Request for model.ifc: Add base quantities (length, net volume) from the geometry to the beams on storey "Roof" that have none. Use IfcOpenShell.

First a look at what the model holds.

```python
import ifcopenshell
import ifcopenshell.util.element
import ifcopenshell.util.unit

model = ifcopenshell.open("model.ifc")
print(model.schema)
for unit_type in ("LENGTHUNIT", "AREAUNIT", "VOLUMEUNIT"):
    print(unit_type, ifcopenshell.util.unit.calculate_unit_scale(model, unit_type))
storey = next(s for s in model.by_type("IfcBuildingStorey") if s.Name == "Roof")
beams = [e for e in ifcopenshell.util.element.get_decomposition(storey) if e.is_a("IfcBeam")]
for e in sorted(beams, key=lambda e: e.id()):
    print(e.id(), e.is_a(), e.Name, list(ifcopenshell.util.element.get_psets(e, qtos_only=True)), sep=" | ")
```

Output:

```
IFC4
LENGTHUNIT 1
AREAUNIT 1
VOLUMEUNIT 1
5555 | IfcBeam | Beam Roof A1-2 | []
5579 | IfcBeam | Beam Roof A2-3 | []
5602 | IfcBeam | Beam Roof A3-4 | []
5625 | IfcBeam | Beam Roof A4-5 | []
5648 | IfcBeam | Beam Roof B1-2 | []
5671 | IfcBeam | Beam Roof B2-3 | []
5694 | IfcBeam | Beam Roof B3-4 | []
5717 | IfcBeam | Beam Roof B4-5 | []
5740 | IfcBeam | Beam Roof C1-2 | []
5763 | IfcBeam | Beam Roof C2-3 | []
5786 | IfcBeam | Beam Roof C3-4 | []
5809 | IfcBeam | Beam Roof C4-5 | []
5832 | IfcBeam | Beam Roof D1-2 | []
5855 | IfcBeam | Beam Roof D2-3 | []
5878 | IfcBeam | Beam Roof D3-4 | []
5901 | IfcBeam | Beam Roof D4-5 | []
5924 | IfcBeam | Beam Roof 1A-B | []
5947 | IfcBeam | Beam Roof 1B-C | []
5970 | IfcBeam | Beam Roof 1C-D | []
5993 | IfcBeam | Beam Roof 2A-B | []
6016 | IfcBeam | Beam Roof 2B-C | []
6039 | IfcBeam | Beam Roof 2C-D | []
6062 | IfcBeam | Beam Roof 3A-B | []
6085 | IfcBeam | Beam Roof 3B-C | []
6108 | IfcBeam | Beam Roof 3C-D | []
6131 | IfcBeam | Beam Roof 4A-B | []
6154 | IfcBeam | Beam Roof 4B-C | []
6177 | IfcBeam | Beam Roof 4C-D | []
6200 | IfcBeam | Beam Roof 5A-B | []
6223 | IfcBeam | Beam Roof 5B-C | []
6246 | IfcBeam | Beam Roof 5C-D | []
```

```python
import ifcopenshell
import ifcopenshell.api.pset
import ifcopenshell.geom
import ifcopenshell.util.element
import ifcopenshell.util.shape
import ifcopenshell.util.unit

model = ifcopenshell.open("model.ifc")
unit_scale = ifcopenshell.util.unit.calculate_unit_scale(model)
volume_scale = ifcopenshell.util.unit.calculate_unit_scale(model, "VOLUMEUNIT")
settings = ifcopenshell.geom.settings()

storey = next(s for s in model.by_type("IfcBuildingStorey") if s.Name == "Roof")
beams = [e for e in ifcopenshell.util.element.get_decomposition(storey) if e.is_a("IfcBeam")]

for e in sorted(beams, key=lambda e: e.id()):
    if ifcopenshell.util.element.get_psets(e, qtos_only=True, should_inherit=False):
        continue
    # Geometry comes back in metres, in the element's own axes.
    shape = ifcopenshell.geom.create_shape(settings, e)
    values = {
        "Length": ifcopenshell.util.shape.get_max_xyz(shape.geometry) / unit_scale,
        "NetVolume": ifcopenshell.util.shape.get_volume(shape.geometry) / volume_scale,
    }
    qto = ifcopenshell.api.pset.add_qto(model, product=e, name="Qto_BeamBaseQuantities")
    ifcopenshell.api.pset.edit_qto(model, qto=qto, properties=values)
    print(e.id(), {k: round(v, 3) for k, v in values.items()})

model.write("model_v2.ifc")
```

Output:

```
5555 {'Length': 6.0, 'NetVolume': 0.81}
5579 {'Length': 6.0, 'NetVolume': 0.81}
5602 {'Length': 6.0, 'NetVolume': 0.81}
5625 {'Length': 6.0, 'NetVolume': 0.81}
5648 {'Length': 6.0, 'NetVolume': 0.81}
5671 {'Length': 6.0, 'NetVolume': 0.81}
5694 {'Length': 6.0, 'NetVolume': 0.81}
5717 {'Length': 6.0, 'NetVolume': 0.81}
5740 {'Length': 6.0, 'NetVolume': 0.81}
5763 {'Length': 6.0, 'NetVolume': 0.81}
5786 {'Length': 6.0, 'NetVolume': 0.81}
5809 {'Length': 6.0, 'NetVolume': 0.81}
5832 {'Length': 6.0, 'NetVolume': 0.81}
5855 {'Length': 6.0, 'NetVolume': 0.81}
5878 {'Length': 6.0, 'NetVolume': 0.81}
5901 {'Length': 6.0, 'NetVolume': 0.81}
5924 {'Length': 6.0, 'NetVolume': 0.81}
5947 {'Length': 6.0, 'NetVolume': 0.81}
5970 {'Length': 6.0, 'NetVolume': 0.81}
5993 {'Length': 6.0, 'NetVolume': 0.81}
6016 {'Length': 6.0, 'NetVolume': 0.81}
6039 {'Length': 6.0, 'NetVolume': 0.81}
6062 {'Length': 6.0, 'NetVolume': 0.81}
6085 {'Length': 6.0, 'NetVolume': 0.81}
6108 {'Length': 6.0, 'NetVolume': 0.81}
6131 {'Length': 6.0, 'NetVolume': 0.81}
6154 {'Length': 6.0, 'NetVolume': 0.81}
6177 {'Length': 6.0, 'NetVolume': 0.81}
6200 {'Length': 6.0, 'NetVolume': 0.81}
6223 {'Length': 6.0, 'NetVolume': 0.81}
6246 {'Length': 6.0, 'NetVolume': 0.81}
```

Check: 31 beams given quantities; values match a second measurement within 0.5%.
